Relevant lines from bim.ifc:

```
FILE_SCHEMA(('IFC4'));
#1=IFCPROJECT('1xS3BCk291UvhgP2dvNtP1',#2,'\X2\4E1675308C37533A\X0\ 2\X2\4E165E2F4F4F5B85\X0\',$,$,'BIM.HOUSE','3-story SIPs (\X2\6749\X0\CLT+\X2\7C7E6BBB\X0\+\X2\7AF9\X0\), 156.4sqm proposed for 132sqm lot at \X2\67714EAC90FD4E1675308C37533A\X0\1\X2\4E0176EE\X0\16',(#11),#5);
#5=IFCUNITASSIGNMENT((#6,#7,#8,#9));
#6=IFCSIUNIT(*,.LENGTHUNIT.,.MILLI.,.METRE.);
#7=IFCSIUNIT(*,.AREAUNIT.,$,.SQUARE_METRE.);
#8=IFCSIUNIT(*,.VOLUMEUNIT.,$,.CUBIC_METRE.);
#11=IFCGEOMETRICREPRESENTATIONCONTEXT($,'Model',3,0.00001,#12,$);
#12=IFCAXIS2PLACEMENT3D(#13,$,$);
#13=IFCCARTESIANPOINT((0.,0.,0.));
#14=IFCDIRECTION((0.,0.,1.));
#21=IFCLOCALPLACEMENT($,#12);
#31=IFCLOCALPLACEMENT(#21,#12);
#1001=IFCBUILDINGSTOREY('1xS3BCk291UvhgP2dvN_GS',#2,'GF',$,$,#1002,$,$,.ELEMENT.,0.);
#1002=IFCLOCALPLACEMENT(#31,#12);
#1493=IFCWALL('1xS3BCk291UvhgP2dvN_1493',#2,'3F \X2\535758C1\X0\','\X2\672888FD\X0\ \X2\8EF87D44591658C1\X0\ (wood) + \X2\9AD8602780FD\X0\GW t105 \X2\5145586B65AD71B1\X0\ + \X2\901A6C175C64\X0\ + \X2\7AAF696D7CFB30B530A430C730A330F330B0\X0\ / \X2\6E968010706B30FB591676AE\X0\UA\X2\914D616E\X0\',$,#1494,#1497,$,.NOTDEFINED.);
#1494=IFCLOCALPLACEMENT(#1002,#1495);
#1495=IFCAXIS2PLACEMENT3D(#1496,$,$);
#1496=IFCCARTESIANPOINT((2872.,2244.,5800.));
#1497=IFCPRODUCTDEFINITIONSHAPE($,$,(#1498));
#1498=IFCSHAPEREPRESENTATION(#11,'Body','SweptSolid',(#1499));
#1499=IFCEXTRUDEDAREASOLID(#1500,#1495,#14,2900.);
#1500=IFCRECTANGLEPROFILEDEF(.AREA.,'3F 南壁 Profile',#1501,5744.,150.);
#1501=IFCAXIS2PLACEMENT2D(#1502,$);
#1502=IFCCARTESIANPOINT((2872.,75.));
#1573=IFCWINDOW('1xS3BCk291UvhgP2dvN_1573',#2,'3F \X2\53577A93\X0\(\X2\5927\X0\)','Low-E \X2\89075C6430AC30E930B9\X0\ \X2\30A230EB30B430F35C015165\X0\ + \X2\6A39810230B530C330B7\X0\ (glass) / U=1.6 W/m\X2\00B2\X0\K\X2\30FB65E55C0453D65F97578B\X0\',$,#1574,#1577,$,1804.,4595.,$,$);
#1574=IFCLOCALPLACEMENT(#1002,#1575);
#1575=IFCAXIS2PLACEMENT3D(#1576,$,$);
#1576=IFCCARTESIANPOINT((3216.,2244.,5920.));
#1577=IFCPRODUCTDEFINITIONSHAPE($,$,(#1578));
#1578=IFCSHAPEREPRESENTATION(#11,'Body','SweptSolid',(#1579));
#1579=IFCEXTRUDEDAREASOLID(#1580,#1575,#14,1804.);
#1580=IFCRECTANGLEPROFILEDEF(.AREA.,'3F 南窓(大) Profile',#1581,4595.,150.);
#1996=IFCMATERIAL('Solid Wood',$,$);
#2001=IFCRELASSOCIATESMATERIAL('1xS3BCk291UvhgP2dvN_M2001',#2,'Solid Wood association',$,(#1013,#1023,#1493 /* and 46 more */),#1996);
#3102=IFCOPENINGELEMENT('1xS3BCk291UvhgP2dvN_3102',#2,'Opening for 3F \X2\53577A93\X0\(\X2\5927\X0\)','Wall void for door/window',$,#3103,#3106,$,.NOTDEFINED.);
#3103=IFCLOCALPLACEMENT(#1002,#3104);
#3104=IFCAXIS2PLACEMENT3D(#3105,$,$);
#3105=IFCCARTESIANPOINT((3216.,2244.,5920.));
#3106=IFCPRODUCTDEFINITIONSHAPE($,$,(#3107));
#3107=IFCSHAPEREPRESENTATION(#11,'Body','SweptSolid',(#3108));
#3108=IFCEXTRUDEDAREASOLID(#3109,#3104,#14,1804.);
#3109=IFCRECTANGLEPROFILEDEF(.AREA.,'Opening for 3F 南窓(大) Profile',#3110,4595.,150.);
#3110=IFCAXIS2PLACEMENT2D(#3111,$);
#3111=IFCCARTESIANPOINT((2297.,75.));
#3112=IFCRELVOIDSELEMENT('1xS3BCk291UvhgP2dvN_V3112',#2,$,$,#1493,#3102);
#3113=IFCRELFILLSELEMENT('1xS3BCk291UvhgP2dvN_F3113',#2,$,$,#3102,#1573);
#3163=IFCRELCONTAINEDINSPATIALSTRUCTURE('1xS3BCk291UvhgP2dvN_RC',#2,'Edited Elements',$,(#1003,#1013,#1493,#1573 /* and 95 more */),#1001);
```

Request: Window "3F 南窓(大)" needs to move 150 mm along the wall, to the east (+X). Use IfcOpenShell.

```python
import ifcopenshell
import ifcopenshell.api.geometry
import ifcopenshell.util.placement

model = ifcopenshell.open("bim.ifc")

window = model.by_guid("1xS3BCk291UvhgP2dvN_1573")
opening = window.FillsVoids[0].RelatingOpeningElement
wall = opening.VoidsElements[0].RelatingBuildingElement

wall_matrix = ifcopenshell.util.placement.get_local_placement(wall.ObjectPlacement)
shift = wall_matrix[:3, 0] * 150.0
before = ifcopenshell.util.placement.get_local_placement(window.ObjectPlacement)[:3, 3].copy()

# The window is not placed relative to its opening, so move both.
for product in (opening, window):
    matrix = ifcopenshell.util.placement.get_local_placement(product.ObjectPlacement)
    matrix[:3, 3] += shift
    ifcopenshell.api.geometry.edit_object_placement(model, product=product, matrix=matrix, is_si=False)

after = ifcopenshell.util.placement.get_local_placement(window.ObjectPlacement)[:3, 3]
print("window moved by", (after - before).round(3) + 0.0)

model.write("bim_rev.ifc")
```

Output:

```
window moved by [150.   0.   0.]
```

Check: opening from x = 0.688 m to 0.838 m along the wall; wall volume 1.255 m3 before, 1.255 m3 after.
